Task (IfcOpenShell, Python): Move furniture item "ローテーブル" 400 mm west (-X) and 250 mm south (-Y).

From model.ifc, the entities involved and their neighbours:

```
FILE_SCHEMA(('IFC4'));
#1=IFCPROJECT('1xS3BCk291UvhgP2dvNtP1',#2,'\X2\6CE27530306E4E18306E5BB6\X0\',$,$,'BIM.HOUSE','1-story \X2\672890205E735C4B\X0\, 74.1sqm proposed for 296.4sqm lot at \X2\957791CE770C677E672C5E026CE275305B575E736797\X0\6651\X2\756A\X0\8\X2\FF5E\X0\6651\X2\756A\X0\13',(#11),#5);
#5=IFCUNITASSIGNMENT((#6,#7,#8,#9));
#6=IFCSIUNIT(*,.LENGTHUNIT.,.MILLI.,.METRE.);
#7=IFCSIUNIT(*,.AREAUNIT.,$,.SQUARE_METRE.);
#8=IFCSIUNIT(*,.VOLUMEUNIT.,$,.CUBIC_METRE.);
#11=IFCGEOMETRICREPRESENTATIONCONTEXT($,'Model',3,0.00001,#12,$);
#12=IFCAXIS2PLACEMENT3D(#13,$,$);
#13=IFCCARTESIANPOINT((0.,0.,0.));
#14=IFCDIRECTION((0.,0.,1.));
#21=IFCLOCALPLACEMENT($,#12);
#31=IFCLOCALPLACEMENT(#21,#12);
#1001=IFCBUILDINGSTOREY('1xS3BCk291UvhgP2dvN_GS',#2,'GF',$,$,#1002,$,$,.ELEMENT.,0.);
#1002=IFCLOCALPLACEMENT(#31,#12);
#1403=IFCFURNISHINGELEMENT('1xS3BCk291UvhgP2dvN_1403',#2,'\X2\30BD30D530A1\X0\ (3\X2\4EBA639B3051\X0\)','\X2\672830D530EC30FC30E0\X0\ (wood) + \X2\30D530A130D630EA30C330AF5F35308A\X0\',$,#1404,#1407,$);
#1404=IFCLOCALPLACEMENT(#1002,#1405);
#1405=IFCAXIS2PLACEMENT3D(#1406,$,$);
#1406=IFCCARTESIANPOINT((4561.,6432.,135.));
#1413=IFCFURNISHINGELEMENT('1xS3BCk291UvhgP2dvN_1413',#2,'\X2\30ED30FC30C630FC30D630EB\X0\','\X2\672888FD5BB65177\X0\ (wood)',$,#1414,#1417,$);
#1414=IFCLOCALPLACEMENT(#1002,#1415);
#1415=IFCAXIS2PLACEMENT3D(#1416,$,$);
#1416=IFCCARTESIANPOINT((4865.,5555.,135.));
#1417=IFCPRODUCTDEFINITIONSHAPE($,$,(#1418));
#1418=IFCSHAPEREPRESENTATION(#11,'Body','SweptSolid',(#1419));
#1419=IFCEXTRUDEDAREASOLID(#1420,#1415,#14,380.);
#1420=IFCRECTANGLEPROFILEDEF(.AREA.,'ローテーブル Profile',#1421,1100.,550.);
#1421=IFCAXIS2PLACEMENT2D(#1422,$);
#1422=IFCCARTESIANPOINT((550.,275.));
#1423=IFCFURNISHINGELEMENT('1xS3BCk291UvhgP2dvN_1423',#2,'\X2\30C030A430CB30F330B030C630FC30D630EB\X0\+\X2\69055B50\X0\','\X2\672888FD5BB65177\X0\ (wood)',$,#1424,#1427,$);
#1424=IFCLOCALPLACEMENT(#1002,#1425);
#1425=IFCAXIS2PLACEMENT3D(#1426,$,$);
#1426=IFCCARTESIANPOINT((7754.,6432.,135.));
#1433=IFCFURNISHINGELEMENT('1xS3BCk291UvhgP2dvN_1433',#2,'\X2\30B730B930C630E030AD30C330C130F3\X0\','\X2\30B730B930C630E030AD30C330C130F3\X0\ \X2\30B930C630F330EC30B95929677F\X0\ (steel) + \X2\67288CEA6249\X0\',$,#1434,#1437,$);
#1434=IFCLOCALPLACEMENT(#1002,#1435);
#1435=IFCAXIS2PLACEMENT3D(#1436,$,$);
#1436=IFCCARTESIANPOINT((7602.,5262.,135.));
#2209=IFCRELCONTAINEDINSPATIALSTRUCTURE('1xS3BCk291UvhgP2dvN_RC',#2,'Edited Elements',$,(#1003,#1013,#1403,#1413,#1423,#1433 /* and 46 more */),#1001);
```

```python
import ifcopenshell
import ifcopenshell.api.geometry
import ifcopenshell.util.placement

model = ifcopenshell.open("model.ifc")

item = model.by_guid("1xS3BCk291UvhgP2dvN_1413")
matrix = ifcopenshell.util.placement.get_local_placement(item.ObjectPlacement)
matrix[0, 3] -= 400.0
matrix[1, 3] -= 250.0
ifcopenshell.api.geometry.edit_object_placement(model, product=item, matrix=matrix, is_si=False)

print(ifcopenshell.util.placement.get_local_placement(item.ObjectPlacement).round(3) + 0.0)

model.write("model_updated.ifc")
```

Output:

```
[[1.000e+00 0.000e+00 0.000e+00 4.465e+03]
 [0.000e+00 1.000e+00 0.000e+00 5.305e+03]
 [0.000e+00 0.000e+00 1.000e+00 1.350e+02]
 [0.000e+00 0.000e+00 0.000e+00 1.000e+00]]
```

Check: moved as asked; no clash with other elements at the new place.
